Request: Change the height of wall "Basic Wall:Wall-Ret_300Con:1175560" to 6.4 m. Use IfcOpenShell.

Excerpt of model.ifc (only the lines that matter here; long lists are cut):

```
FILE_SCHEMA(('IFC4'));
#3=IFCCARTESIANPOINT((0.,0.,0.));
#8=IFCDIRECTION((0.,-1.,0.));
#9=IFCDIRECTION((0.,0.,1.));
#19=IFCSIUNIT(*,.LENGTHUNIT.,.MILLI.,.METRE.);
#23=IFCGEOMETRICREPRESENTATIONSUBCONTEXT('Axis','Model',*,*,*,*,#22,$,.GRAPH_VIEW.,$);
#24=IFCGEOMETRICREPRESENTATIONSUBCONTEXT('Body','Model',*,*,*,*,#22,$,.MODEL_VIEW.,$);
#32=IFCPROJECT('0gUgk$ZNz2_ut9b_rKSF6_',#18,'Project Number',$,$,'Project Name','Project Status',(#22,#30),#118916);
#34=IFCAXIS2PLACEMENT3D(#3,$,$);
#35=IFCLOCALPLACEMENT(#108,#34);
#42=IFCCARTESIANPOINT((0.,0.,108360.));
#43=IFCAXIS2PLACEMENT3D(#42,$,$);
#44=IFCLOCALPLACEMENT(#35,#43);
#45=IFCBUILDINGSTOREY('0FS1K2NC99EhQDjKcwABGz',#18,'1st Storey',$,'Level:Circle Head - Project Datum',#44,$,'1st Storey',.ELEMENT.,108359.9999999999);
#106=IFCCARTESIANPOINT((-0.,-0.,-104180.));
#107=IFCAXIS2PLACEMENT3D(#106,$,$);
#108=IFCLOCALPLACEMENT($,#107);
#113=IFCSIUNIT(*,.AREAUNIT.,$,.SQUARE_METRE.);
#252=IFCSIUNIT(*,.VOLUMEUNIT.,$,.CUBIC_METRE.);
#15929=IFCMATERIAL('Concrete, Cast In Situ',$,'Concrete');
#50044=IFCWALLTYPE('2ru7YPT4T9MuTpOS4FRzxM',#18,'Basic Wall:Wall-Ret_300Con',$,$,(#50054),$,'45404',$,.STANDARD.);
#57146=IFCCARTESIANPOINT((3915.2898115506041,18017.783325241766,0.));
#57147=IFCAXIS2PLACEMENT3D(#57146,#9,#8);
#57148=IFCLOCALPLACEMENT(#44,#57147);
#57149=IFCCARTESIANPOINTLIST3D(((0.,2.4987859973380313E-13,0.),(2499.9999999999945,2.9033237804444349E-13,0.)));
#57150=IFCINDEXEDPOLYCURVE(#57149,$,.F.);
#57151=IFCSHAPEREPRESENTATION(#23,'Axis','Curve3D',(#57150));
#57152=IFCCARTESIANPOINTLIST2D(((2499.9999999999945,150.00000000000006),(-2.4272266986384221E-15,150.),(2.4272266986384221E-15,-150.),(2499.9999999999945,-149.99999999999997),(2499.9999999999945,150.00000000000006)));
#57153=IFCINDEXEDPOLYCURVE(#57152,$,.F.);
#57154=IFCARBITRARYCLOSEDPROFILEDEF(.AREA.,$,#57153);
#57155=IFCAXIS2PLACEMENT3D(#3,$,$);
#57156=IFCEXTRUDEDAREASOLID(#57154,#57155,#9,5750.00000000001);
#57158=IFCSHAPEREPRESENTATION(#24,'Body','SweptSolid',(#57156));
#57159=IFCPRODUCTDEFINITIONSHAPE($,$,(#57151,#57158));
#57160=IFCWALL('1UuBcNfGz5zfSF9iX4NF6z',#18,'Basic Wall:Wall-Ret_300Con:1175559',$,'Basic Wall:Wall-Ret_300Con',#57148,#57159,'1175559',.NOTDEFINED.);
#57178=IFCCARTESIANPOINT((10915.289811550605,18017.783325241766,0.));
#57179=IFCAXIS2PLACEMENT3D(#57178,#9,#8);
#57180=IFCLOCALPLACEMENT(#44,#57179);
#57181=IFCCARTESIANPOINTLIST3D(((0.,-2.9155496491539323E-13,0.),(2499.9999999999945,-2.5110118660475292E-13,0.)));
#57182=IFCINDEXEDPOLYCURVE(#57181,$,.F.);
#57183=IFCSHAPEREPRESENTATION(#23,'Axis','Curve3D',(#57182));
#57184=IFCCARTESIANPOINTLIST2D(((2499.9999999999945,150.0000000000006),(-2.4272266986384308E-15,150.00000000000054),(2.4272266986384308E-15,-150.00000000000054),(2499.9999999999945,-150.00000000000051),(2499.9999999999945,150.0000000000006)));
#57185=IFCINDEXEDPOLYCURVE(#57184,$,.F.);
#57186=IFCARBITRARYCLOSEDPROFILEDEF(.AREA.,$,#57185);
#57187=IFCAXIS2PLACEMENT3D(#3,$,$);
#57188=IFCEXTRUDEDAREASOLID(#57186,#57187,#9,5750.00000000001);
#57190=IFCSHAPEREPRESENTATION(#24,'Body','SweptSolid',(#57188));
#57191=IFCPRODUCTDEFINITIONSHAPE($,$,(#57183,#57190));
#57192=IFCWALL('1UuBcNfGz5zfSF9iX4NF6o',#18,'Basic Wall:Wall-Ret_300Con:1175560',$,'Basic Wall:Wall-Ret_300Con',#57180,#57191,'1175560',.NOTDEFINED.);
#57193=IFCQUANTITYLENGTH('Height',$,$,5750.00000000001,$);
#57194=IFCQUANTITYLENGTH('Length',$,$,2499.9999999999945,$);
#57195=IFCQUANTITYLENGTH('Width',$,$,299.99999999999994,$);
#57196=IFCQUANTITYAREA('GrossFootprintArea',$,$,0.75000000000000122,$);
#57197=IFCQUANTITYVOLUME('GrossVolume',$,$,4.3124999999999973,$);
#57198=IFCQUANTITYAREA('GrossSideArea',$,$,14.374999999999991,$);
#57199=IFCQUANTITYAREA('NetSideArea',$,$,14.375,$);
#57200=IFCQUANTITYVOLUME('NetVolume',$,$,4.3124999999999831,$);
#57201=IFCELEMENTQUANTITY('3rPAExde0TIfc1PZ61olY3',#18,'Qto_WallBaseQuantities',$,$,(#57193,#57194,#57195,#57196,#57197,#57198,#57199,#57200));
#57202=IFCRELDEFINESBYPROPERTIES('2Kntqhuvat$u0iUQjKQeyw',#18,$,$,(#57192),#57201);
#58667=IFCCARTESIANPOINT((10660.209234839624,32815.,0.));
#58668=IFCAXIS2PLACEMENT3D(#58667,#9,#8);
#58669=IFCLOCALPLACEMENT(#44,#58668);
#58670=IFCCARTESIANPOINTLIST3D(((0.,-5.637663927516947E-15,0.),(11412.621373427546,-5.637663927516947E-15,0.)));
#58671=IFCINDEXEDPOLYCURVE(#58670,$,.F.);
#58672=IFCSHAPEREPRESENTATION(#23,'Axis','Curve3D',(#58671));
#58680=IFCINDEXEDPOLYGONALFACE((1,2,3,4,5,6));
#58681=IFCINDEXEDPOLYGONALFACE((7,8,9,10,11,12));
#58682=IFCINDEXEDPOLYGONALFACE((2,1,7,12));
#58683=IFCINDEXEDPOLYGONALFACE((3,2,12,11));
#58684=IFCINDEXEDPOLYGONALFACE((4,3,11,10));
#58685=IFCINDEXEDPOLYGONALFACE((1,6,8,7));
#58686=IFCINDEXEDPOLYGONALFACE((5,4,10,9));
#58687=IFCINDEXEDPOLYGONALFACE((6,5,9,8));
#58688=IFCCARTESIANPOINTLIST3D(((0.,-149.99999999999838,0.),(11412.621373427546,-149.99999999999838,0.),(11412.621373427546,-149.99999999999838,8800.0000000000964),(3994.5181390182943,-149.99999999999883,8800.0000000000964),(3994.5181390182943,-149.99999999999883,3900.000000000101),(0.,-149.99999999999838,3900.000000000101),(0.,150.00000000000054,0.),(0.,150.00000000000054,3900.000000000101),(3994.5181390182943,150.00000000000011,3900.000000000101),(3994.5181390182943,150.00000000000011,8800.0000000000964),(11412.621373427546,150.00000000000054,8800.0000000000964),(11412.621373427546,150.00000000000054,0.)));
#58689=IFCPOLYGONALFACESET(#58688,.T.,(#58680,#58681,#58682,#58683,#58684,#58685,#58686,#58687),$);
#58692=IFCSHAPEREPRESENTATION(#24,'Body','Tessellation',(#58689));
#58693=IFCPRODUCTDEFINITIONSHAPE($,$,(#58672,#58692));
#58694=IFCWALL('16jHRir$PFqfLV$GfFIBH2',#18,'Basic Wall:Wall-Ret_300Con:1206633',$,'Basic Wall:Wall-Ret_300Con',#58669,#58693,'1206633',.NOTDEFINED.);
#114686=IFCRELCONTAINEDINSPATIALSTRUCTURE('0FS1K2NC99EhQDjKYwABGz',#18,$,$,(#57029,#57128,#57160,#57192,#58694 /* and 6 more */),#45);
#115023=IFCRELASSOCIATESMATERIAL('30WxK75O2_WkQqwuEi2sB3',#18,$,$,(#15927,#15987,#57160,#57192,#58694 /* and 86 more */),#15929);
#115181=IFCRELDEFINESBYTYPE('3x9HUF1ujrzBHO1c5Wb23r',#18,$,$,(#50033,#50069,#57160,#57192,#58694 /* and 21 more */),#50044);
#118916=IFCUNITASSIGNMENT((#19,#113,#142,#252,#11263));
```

```python
import ifcopenshell
import ifcopenshell.api.pset
import ifcopenshell.geom
import ifcopenshell.util.element
import ifcopenshell.util.representation
import ifcopenshell.util.shape
import ifcopenshell.util.unit

model = ifcopenshell.open("model.ifc")
unit_scale = ifcopenshell.util.unit.calculate_unit_scale(model)
area_scale = ifcopenshell.util.unit.calculate_unit_scale(model, "AREAUNIT")
volume_scale = ifcopenshell.util.unit.calculate_unit_scale(model, "VOLUMEUNIT")
settings = ifcopenshell.geom.settings()


def volume(element):
    """Net volume in cubic metres, openings subtracted."""
    shape = ifcopenshell.geom.create_shape(settings, element)
    return ifcopenshell.util.shape.get_volume(shape.geometry)


wall = model.by_guid("1UuBcNfGz5zfSF9iX4NF6o")
before = volume(wall)

body = ifcopenshell.util.representation.get_representation(wall, "Model", "Body")
solid = body.Items[0]
old_height = solid.Depth
solid.Depth = 6.4 / unit_scale
after = volume(wall)
thickness = 0.3  # wall thickness in metres

# Update the stored height, areas and volumes.
qto = model.by_id(ifcopenshell.util.element.get_pset(wall, "Qto_WallBaseQuantities", should_inherit=False)["id"])
ifcopenshell.api.pset.edit_qto(model, qto=qto, properties={
    "Height": solid.Depth,
    "GrossVolume": ifcopenshell.util.element.get_pset(wall, "Qto_WallBaseQuantities", "GrossVolume") * solid.Depth / old_height,
    "GrossSideArea": ifcopenshell.util.element.get_pset(wall, "Qto_WallBaseQuantities", "GrossSideArea") * solid.Depth / old_height,
    "NetSideArea": after / thickness / area_scale,
    "NetVolume": after / volume_scale,
})

print(f"height {old_height:g} -> {solid.Depth:g}, volume {before:.3f} -> {after:.3f} m3")

model.write("model_rev.ifc")
```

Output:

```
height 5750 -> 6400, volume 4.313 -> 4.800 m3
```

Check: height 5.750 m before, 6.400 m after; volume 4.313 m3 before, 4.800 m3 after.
